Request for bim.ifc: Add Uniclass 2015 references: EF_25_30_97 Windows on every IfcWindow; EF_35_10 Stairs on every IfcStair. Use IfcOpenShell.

First a look at what the model holds.

```python
import ifcopenshell

model = ifcopenshell.open("bim.ifc")
print(model.schema)
print("classifications:", [c.Name for c in model.by_type("IfcClassification")])
for ifc_class in ("IfcDoor", "IfcRoof", "IfcStair", "IfcWall", "IfcWindow"):
    print(ifc_class, len(model.by_type(ifc_class)))
```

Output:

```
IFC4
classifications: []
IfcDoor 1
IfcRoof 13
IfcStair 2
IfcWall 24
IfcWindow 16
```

```python
import ifcopenshell
import ifcopenshell.api.classification

model = ifcopenshell.open("bim.ifc")

system = ifcopenshell.api.classification.add_classification(model, classification="Uniclass 2015")

codes = {
    "IfcWindow": ("EF_25_30_97", "Windows"),
    "IfcStair": ("EF_35_10", "Stairs"),
}
for ifc_class, (code, name) in codes.items():
    products = model.by_type(ifc_class)
    ifcopenshell.api.classification.add_reference(
        model, products=products, classification=system, identification=code, name=name
    )
    print(code, len(products))

model.write("bim-out.ifc")
```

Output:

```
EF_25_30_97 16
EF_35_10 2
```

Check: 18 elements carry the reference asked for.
